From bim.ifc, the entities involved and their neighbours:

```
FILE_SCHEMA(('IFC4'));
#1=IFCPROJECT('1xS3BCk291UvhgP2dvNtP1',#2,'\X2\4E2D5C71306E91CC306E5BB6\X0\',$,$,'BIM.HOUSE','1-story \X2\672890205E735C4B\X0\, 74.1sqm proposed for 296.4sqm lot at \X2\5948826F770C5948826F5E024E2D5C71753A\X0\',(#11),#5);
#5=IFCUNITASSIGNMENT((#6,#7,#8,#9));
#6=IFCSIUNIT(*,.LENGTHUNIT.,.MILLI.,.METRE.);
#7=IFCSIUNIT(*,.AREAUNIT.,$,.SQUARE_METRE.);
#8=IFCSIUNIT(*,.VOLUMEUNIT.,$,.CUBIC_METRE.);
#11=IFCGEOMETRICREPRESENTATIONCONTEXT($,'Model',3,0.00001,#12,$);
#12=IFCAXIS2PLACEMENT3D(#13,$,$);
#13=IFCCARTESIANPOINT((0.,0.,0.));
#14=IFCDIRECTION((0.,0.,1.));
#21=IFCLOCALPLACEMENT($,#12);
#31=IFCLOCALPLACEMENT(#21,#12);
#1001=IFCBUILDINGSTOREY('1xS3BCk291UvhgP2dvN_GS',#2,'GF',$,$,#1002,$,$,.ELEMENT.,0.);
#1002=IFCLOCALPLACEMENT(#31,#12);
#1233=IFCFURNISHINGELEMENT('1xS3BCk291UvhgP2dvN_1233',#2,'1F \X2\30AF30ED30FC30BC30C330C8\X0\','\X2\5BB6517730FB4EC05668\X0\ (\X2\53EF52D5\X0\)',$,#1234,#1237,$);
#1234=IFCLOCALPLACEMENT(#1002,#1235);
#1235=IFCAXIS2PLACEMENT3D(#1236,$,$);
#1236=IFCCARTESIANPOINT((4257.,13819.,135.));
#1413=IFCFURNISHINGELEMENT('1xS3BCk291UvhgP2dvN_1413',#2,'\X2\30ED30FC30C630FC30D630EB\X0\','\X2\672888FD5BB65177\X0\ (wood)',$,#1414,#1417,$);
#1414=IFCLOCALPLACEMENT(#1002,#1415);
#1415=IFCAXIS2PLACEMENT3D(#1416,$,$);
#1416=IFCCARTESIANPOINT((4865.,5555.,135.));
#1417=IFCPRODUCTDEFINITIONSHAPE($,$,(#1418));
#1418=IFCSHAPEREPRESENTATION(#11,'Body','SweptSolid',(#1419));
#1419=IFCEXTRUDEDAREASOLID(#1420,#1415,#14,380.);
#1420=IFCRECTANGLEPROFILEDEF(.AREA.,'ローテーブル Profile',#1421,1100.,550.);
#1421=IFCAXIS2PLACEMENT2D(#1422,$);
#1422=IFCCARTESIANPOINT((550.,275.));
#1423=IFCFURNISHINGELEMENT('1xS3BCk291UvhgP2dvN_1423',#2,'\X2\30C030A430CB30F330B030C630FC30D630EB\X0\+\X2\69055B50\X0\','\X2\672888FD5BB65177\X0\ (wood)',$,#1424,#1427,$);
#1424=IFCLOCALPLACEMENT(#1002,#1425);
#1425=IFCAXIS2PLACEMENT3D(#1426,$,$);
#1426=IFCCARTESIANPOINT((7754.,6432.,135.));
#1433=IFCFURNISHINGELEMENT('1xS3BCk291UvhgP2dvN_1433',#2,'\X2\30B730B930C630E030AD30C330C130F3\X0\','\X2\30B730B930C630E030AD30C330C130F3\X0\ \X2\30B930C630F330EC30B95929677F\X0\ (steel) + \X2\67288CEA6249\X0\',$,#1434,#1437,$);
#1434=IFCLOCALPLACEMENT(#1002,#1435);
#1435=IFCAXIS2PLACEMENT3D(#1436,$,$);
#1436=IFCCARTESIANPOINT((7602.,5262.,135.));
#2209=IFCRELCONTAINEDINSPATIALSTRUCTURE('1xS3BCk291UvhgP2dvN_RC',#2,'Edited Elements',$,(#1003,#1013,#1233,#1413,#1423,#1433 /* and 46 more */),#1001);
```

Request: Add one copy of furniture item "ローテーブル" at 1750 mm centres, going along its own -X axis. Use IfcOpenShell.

```python
import ifcopenshell
import ifcopenshell.api.geometry
import ifcopenshell.api.root
import ifcopenshell.util.element
import ifcopenshell.util.placement
import ifcopenshell.util.unit

model = ifcopenshell.open("bim.ifc")
unit_scale = ifcopenshell.util.unit.calculate_unit_scale(model)


def reuse_history(source, copy):
    """copy_class also copies each property set's owner history, people and application; keep the originals."""
    for rel in copy.IsDefinedBy:
        if rel.is_a("IfcRelDefinesByProperties") and (history := rel.RelatingPropertyDefinition.OwnerHistory):
            rel.RelatingPropertyDefinition.OwnerHistory = source.OwnerHistory
            ifcopenshell.util.element.remove_deep2(model, history)


source = model.by_guid("1xS3BCk291UvhgP2dvN_1413")
base = ifcopenshell.util.placement.get_local_placement(source.ObjectPlacement)
step = -base[:3, 0] * 1.75 / unit_scale

for i in range(1, 2):
    copy = ifcopenshell.api.root.copy_class(model, product=source)
    copy.Representation = ifcopenshell.util.element.copy_deep(
        model, source.Representation, exclude=["IfcGeometricRepresentationContext", "IfcRepresentationMap"]
    )
    reuse_history(source, copy)
    matrix = base.copy()
    matrix[:3, 3] += i * step
    print("added at", matrix[:3, 3].round(3) + 0.0)
    ifcopenshell.api.geometry.edit_object_placement(model, product=copy, matrix=matrix, is_si=False)

model.write("bim_v2.ifc")
```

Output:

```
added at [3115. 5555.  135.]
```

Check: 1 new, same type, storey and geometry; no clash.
